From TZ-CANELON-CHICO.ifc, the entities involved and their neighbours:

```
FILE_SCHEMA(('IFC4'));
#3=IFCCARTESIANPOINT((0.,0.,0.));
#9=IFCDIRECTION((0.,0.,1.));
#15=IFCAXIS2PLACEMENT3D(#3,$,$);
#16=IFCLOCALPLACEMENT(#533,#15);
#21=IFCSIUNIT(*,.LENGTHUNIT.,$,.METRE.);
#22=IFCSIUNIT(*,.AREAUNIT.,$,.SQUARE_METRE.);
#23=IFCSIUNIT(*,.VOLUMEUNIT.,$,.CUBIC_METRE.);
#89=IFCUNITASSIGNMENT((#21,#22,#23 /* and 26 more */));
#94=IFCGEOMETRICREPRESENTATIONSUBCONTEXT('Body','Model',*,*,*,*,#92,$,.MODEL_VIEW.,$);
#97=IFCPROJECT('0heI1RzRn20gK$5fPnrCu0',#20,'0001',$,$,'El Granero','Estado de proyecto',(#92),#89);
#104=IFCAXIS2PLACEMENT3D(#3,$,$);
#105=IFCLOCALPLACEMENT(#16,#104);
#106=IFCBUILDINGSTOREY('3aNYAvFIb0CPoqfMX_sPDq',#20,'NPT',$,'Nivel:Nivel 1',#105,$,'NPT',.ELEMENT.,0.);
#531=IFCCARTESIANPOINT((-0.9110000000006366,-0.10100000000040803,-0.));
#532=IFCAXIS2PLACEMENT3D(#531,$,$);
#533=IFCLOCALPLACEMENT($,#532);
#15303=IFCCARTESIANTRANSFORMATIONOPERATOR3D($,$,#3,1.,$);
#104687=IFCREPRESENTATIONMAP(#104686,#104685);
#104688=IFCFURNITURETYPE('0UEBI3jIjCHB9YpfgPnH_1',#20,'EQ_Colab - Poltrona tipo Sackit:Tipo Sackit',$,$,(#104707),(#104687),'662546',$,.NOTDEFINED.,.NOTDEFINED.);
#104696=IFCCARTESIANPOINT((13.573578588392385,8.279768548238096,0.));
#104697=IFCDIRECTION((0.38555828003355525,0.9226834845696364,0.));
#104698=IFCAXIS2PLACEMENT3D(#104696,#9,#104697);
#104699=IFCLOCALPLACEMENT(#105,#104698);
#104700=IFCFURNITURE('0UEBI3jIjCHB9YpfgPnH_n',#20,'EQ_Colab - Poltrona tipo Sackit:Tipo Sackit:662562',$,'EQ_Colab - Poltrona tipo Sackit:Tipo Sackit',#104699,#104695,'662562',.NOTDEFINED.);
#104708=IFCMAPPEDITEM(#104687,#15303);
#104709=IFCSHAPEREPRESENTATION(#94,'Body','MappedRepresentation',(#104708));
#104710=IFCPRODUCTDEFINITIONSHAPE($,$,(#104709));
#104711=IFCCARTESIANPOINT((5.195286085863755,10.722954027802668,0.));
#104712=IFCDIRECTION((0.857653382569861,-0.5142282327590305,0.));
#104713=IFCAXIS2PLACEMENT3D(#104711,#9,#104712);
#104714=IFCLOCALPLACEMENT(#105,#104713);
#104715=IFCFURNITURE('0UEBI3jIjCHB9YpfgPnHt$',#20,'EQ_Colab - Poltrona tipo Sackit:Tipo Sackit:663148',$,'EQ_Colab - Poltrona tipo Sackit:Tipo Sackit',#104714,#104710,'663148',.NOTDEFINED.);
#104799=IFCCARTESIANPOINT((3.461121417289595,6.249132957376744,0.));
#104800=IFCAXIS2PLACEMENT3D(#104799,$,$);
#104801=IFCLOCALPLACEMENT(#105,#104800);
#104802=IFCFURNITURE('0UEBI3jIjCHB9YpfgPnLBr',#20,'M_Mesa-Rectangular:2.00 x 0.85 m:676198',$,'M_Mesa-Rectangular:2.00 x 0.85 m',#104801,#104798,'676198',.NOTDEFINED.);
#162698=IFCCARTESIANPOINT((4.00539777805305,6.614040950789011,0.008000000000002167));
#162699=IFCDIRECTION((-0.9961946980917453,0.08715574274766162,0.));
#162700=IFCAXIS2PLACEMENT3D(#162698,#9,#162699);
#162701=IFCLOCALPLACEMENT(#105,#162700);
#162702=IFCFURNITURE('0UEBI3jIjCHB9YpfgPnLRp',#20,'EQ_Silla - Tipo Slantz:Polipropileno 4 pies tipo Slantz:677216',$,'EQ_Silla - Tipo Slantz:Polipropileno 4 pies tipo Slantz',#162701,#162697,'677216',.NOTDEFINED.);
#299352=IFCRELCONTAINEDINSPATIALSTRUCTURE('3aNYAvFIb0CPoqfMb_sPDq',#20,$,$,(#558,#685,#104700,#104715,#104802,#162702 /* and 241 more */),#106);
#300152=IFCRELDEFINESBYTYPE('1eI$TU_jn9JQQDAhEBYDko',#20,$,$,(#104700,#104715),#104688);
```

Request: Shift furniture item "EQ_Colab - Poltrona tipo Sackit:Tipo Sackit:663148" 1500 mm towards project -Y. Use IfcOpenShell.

```python
import ifcopenshell
import ifcopenshell.api.geometry
import ifcopenshell.util.placement
import ifcopenshell.util.unit

model = ifcopenshell.open("TZ-CANELON-CHICO.ifc")
unit_scale = ifcopenshell.util.unit.calculate_unit_scale(model)

item = model.by_id(104715)
matrix = ifcopenshell.util.placement.get_local_placement(item.ObjectPlacement)
matrix[1, 3] -= 1.5 / unit_scale
ifcopenshell.api.geometry.edit_object_placement(model, product=item, matrix=matrix, is_si=False)

print(ifcopenshell.util.placement.get_local_placement(item.ObjectPlacement).round(3) + 0.0)

model.write("TZ-CANELON-CHICO_updated.ifc")
```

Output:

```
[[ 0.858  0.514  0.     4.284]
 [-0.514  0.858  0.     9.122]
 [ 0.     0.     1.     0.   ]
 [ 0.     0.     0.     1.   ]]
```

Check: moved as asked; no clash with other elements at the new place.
